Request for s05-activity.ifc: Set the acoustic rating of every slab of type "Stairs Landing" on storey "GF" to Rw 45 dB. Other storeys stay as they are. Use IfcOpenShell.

First a look at what the model holds.

```python
import ifcopenshell
import ifcopenshell.util.element

model = ifcopenshell.open("s05-activity.ifc")
print(model.schema)
storey = next(s for s in model.by_type("IfcBuildingStorey") if s.Name == "GF")
slabs = [e for e in ifcopenshell.util.element.get_decomposition(storey) if e.is_a("IfcSlab")]
seen = {}
for e in slabs:
    element_type = ifcopenshell.util.element.get_type(e)
    key = (element_type.Name if element_type != e and element_type else None, ifcopenshell.util.element.get_pset(e, "Pset_SlabCommon", "AcousticRating"))
    seen[key] = seen.get(key, 0) + 1
for (name, value), count in sorted(seen.items(), key=str):
    print(count, "x", name, "|", value)
```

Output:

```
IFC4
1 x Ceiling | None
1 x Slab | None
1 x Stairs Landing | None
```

```python
import ifcopenshell
import ifcopenshell.api.pset
import ifcopenshell.util.element

model = ifcopenshell.open("s05-activity.ifc")

storey = next(s for s in model.by_type("IfcBuildingStorey") if s.Name == "GF")
slabs = [e for e in ifcopenshell.util.element.get_decomposition(storey) if e.is_a("IfcSlab")]

count = 0
for e in slabs:
    element_type = ifcopenshell.util.element.get_type(e)
    if element_type in (None, e) or element_type.Name != "Stairs Landing":
        continue
    # add_pset returns the element's existing set when there is one.
    pset = ifcopenshell.api.pset.add_pset(model, product=e, name="Pset_SlabCommon")
    ifcopenshell.api.pset.edit_pset(model, pset=pset, properties={"AcousticRating": "Rw 45 dB"})
    count += 1

print(count, "slabs updated")

model.write("s05-activity_updated.ifc")
```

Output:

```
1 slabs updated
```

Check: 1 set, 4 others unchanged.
